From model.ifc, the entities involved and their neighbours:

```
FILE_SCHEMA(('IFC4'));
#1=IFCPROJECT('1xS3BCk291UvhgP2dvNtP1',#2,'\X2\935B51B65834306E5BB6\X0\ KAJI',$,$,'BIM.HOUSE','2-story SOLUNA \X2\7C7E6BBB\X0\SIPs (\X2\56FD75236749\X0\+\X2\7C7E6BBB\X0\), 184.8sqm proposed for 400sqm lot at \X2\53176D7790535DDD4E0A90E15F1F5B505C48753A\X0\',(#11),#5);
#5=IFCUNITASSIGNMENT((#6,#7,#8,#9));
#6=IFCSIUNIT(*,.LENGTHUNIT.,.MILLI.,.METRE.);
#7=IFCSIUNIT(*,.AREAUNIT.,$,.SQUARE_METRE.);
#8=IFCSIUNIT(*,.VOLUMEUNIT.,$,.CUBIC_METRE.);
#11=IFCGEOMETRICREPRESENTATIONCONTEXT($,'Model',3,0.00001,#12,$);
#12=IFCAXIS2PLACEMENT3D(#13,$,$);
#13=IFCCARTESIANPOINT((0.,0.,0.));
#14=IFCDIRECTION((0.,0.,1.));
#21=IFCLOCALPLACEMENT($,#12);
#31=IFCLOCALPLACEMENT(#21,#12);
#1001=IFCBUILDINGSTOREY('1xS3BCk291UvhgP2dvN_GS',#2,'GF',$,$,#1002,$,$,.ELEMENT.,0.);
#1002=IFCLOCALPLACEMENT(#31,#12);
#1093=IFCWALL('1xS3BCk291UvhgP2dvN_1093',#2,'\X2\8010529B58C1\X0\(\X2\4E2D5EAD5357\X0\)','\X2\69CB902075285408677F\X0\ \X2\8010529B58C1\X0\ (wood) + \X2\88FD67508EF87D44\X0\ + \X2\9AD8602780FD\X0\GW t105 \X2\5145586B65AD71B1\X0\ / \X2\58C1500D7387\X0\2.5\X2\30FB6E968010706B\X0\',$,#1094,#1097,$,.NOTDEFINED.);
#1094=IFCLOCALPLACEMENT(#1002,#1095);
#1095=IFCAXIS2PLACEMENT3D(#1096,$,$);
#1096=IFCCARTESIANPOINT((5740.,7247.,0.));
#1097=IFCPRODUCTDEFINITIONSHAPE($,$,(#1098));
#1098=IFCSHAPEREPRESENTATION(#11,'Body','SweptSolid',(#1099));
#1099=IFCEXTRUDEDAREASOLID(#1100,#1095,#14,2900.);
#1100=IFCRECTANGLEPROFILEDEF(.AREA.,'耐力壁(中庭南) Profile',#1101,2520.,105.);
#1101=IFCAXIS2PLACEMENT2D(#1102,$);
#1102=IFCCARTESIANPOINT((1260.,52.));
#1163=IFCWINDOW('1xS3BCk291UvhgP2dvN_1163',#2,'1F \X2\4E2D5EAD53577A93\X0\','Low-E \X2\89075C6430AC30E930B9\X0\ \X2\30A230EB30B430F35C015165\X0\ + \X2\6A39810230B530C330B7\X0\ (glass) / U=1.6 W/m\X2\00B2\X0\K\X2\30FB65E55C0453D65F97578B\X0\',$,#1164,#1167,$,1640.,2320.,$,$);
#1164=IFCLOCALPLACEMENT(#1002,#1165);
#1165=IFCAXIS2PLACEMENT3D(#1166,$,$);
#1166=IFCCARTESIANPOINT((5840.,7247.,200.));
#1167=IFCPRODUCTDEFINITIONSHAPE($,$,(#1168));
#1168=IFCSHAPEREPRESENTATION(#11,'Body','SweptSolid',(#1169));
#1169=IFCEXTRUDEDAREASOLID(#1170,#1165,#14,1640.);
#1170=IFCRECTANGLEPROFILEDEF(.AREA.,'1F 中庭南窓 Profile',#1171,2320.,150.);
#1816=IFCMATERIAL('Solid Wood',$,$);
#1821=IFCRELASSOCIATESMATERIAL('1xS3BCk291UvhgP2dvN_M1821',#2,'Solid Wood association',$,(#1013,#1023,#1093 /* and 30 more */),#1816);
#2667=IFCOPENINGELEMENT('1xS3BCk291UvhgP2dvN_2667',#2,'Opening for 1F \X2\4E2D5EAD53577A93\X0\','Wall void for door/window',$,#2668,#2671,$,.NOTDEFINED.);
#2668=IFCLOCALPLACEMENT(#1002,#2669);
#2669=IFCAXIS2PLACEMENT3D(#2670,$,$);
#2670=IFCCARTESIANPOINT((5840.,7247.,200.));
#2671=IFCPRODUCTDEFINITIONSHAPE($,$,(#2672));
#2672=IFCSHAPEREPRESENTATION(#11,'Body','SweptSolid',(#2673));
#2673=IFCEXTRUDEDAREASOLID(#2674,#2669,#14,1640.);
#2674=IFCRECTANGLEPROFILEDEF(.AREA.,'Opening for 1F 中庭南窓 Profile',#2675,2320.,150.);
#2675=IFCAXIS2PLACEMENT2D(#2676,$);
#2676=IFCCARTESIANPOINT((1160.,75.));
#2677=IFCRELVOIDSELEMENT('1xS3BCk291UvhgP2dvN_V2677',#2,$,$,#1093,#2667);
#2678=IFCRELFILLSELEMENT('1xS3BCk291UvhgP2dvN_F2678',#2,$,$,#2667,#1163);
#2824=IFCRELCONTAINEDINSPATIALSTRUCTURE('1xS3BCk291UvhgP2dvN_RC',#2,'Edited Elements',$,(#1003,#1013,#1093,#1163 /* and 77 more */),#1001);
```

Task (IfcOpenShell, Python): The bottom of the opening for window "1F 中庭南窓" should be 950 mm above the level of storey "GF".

```python
import numpy as np
import ifcopenshell
import ifcopenshell.api.geometry
import ifcopenshell.geom
import ifcopenshell.util.element
import ifcopenshell.util.placement
import ifcopenshell.util.shape
import ifcopenshell.util.unit

model = ifcopenshell.open("model.ifc")
unit_scale = ifcopenshell.util.unit.calculate_unit_scale(model)

window = model.by_guid("1xS3BCk291UvhgP2dvN_1163")
opening = window.FillsVoids[0].RelatingOpeningElement
storey = ifcopenshell.util.element.get_container(window, ifc_class="IfcBuildingStorey")
level = ifcopenshell.util.placement.get_local_placement(storey.ObjectPlacement)[2, 3]

# The opening's origin need not be at the sill, so measure its lowest point.
shape = ifcopenshell.geom.create_shape(ifcopenshell.geom.settings(), opening)
bottom = ifcopenshell.util.shape.get_shape_bottom_elevation(shape, shape.geometry) / unit_scale
dz = level + 950.0 - bottom

shift = np.array([0.0, 0.0, dz])
# The window is not placed relative to its opening, so move both.
for product in (opening, window):
    matrix = ifcopenshell.util.placement.get_local_placement(product.ObjectPlacement)
    matrix[:3, 3] += shift
    ifcopenshell.api.geometry.edit_object_placement(model, product=product, matrix=matrix, is_si=False)

print(f"moved by {dz * unit_scale:+.3f} m")

model.write("model_rev.ifc")
```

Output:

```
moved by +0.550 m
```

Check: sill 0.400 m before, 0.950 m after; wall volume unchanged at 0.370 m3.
